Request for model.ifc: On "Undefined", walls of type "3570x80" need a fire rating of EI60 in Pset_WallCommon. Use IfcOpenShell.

First a look at what the model holds.

```python
import ifcopenshell
import ifcopenshell.util.element

model = ifcopenshell.open("model.ifc")
print(model.schema)
storey = next(s for s in model.by_type("IfcBuildingStorey") if s.Name == "Undefined")
walls = [e for e in ifcopenshell.util.element.get_decomposition(storey) if e.is_a("IfcWall")]
seen = {}
for e in walls:
    element_type = ifcopenshell.util.element.get_type(e)
    key = (element_type.Name if element_type != e and element_type else None, ifcopenshell.util.element.get_pset(e, "Pset_WallCommon", "FireRating"))
    seen[key] = seen.get(key, 0) + 1
for (name, value), count in sorted(seen.items(), key=str):
    print(count, "x", name, "|", value)
```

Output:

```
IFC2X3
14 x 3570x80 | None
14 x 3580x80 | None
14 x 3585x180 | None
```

```python
import ifcopenshell
import ifcopenshell.api.pset
import ifcopenshell.util.element

model = ifcopenshell.open("model.ifc")

storey = next(s for s in model.by_type("IfcBuildingStorey") if s.Name == "Undefined")
walls = [e for e in ifcopenshell.util.element.get_decomposition(storey) if e.is_a("IfcWall")]

count = 0
for e in walls:
    element_type = ifcopenshell.util.element.get_type(e)
    if element_type in (None, e) or element_type.Name != "3570x80":
        continue
    found = ifcopenshell.util.element.get_pset(e, "Pset_WallCommon", should_inherit=False)
    if found:
        pset = model.by_id(found["id"])
        if len(ifcopenshell.util.element.get_elements_by_pset(pset)) > 1:
            pset = ifcopenshell.api.pset.unshare_pset(model, products=[e], pset=pset)[0]
    else:
        pset = ifcopenshell.api.pset.add_pset(model, product=e, name="Pset_WallCommon")
    ifcopenshell.api.pset.edit_pset(model, pset=pset, properties={"FireRating": "EI60"})
    count += 1

print(count, "walls updated")

model.write("model-out.ifc")
```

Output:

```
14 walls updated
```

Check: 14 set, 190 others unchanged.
